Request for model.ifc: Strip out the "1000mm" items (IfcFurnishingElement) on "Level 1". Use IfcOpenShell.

First a look at what the model holds.

```python
import ifcopenshell
import ifcopenshell.util.element

model = ifcopenshell.open("model.ifc")
print(model.schema)
storey = next(s for s in model.by_type("IfcBuildingStorey") if s.Name == "Level 1")
furniture = [e for e in ifcopenshell.util.element.get_decomposition(storey) if e.is_a("IfcFurnishingElement")]
seen = {}
for e in furniture:
    element_type = ifcopenshell.util.element.get_type(e)
    name = element_type.Name if element_type not in (None, e) else None
    seen[name] = seen.get(name, 0) + 1
for name, count in sorted(seen.items(), key=str):
    print(count, "x", name)
```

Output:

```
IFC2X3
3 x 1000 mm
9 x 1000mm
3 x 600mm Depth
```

```python
import ifcopenshell
import ifcopenshell.api.root
import ifcopenshell.util.element

model = ifcopenshell.open("model.ifc")

storey = next(s for s in model.by_type("IfcBuildingStorey") if s.Name == "Level 1")
furniture = [e for e in ifcopenshell.util.element.get_decomposition(storey) if e.is_a("IfcFurnishingElement")]
targets = [e for e in furniture if (t := ifcopenshell.util.element.get_type(e)) not in (None, e) and t.Name == "1000mm"]

for e in targets:
    ifcopenshell.api.root.remove_product(model, product=e)
print(len(targets), "removed")

model.write("model_edited.ifc")
```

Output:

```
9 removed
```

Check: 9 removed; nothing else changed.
